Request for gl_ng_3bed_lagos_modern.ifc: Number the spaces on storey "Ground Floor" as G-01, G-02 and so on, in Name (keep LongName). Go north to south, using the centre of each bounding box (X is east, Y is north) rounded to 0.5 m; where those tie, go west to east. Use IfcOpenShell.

First a look at what the model holds.

```python
import ifcopenshell
import ifcopenshell.util.element
import ifcopenshell.util.placement

model = ifcopenshell.open("gl_ng_3bed_lagos_modern.ifc")
print(model.schema)
storey = next(s for s in model.by_type("IfcBuildingStorey") if s.Name == "Ground Floor")
spaces = [e for e in ifcopenshell.util.element.get_decomposition(storey) if e.is_a("IfcSpace")]
for e in sorted(spaces, key=lambda e: e.id()):
    origin = ifcopenshell.util.placement.get_local_placement(e.ObjectPlacement)[:3, 3]
    print(e.id(), e.Name, e.LongName, origin.round(2) + 0.0, sep=" | ")
```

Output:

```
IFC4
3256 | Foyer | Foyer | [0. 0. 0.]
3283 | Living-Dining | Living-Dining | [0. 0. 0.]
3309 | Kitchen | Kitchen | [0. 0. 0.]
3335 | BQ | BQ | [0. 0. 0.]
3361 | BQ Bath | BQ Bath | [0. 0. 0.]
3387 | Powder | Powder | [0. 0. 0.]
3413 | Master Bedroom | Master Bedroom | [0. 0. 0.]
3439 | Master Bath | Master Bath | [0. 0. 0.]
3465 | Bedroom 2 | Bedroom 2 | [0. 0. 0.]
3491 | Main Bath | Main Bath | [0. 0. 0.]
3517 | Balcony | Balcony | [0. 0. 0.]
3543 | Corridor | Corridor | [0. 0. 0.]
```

```python
import ifcopenshell
import ifcopenshell.geom
import ifcopenshell.util.element
import ifcopenshell.util.shape

model = ifcopenshell.open("gl_ng_3bed_lagos_modern.ifc")
settings = ifcopenshell.geom.settings()
settings.set("use-world-coords", True)


def centre(element):
    shape = ifcopenshell.geom.create_shape(settings, element)
    return ifcopenshell.util.shape.get_bbox_centroid(shape.geometry)


storey = next(s for s in model.by_type("IfcBuildingStorey") if s.Name == "Ground Floor")
spaces = [e for e in ifcopenshell.util.element.get_decomposition(storey) if e.is_a("IfcSpace")]

# Insertion points can sit at a corner or the storey origin, so sort by the geometry (in metres).
centres = {e: centre(e) for e in spaces}
spaces.sort(key=lambda e: (-round(centres[e][1] / 0.5), centres[e][0]))

for i, e in enumerate(spaces, start=1):
    number = f"G-{i:02d}"
    e.Name = number
    print(e.id(), number)

model.write("gl_ng_3bed_lagos_modern_rev.ifc")
```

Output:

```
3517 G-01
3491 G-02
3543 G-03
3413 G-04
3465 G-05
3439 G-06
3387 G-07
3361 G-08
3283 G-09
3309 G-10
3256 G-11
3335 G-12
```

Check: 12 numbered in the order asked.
